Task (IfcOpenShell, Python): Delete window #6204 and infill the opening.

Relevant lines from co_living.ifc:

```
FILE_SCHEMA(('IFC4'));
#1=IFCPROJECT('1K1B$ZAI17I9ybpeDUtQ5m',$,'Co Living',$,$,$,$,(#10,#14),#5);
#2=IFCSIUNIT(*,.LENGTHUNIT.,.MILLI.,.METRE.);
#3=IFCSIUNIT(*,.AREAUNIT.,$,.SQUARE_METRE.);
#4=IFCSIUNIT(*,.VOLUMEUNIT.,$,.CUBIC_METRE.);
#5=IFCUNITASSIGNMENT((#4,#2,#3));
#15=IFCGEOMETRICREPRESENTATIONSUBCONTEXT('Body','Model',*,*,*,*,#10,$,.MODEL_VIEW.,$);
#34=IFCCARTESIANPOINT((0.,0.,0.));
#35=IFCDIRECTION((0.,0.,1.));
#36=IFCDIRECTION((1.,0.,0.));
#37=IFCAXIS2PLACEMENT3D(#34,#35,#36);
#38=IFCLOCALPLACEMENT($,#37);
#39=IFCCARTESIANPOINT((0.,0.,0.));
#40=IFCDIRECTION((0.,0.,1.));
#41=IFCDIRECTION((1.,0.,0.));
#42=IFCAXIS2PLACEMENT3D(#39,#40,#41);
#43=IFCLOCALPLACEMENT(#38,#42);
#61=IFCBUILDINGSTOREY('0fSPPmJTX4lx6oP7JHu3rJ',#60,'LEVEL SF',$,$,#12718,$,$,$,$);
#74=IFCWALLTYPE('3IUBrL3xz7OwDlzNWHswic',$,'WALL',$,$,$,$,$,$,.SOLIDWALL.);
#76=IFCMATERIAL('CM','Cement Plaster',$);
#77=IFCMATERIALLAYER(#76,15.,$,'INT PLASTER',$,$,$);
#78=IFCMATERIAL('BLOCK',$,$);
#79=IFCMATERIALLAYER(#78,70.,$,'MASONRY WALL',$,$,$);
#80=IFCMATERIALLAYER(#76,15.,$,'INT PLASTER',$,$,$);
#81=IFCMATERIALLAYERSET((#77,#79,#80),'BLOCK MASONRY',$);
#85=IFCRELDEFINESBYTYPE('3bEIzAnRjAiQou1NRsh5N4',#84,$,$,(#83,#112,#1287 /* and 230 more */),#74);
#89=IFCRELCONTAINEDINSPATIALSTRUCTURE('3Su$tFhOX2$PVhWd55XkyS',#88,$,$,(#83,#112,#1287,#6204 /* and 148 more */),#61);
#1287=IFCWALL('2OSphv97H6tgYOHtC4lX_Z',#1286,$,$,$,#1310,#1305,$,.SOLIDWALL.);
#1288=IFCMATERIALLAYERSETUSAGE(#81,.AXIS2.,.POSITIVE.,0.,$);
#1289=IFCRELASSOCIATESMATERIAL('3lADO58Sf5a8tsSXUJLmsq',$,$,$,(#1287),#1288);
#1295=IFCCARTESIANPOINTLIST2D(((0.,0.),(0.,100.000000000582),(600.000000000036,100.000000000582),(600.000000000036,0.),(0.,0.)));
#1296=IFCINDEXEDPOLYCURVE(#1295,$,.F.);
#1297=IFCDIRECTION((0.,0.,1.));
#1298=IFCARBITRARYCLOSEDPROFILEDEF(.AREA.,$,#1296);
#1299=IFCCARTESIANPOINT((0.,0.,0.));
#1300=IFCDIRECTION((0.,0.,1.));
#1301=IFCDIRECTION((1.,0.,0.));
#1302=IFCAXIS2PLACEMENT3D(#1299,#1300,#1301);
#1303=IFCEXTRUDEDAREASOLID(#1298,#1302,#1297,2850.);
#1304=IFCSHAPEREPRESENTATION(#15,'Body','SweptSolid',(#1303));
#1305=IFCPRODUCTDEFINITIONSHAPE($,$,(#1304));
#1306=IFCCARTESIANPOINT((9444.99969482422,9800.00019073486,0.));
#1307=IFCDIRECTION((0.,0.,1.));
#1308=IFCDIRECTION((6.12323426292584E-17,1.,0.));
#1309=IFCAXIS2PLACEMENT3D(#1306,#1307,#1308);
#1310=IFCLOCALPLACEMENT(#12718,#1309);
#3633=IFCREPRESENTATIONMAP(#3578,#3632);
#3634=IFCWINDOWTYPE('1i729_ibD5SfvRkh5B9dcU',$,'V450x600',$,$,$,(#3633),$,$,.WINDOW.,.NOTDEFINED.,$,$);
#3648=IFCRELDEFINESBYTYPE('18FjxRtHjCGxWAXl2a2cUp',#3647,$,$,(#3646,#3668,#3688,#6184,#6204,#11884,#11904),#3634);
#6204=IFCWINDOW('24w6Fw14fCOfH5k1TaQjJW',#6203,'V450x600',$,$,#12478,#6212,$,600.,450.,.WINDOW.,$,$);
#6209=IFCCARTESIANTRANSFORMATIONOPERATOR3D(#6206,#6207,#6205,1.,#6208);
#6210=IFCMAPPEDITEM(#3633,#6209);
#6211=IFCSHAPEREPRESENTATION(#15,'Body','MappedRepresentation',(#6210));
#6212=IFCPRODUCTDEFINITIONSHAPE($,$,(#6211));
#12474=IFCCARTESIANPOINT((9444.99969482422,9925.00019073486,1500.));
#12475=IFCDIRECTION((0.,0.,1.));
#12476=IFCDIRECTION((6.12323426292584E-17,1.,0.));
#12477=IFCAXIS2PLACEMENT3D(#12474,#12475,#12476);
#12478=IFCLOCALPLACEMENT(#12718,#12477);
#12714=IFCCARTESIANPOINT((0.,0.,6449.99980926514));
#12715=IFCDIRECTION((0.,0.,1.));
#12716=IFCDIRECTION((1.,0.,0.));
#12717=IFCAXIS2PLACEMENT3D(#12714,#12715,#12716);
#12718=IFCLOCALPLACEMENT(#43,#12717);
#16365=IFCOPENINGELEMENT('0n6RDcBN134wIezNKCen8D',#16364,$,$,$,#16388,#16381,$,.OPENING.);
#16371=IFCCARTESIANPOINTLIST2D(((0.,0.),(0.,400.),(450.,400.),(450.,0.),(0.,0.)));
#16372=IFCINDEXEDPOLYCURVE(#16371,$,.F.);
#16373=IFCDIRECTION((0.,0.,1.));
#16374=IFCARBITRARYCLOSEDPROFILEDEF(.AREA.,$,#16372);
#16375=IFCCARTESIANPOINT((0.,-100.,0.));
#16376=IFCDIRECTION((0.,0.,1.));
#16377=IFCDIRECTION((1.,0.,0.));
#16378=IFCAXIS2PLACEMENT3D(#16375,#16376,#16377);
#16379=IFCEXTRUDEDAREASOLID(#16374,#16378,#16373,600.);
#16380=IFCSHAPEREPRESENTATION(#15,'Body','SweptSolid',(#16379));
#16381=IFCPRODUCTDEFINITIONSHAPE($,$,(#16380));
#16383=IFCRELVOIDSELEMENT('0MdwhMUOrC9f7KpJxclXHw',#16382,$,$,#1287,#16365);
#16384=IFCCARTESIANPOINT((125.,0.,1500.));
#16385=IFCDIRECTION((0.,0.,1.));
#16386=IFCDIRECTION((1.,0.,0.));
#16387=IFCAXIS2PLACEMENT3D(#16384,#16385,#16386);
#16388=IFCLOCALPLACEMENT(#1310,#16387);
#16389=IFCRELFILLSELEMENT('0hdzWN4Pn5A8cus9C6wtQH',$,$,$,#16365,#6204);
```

```python
import ifcopenshell
import ifcopenshell.api.feature
import ifcopenshell.api.root
import ifcopenshell.geom
import ifcopenshell.util.shape

model = ifcopenshell.open("co_living.ifc")
settings = ifcopenshell.geom.settings()


def volume(element):
    """Net volume in cubic metres, openings subtracted."""
    shape = ifcopenshell.geom.create_shape(settings, element)
    return ifcopenshell.util.shape.get_volume(shape.geometry)


window = model.by_guid("24w6Fw14fCOfH5k1TaQjJW")
opening = window.FillsVoids[0].RelatingOpeningElement
wall = opening.VoidsElements[0].RelatingBuildingElement
before = volume(wall)

ifcopenshell.api.root.remove_product(model, product=window)
ifcopenshell.api.feature.remove_feature(model, feature=opening)

after = volume(wall)

print(f"wall volume {before:.3f} -> {after:.3f} m3")

model.write("co_living_edited.ifc")
```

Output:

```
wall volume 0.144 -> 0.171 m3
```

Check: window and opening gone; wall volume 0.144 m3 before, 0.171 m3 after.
